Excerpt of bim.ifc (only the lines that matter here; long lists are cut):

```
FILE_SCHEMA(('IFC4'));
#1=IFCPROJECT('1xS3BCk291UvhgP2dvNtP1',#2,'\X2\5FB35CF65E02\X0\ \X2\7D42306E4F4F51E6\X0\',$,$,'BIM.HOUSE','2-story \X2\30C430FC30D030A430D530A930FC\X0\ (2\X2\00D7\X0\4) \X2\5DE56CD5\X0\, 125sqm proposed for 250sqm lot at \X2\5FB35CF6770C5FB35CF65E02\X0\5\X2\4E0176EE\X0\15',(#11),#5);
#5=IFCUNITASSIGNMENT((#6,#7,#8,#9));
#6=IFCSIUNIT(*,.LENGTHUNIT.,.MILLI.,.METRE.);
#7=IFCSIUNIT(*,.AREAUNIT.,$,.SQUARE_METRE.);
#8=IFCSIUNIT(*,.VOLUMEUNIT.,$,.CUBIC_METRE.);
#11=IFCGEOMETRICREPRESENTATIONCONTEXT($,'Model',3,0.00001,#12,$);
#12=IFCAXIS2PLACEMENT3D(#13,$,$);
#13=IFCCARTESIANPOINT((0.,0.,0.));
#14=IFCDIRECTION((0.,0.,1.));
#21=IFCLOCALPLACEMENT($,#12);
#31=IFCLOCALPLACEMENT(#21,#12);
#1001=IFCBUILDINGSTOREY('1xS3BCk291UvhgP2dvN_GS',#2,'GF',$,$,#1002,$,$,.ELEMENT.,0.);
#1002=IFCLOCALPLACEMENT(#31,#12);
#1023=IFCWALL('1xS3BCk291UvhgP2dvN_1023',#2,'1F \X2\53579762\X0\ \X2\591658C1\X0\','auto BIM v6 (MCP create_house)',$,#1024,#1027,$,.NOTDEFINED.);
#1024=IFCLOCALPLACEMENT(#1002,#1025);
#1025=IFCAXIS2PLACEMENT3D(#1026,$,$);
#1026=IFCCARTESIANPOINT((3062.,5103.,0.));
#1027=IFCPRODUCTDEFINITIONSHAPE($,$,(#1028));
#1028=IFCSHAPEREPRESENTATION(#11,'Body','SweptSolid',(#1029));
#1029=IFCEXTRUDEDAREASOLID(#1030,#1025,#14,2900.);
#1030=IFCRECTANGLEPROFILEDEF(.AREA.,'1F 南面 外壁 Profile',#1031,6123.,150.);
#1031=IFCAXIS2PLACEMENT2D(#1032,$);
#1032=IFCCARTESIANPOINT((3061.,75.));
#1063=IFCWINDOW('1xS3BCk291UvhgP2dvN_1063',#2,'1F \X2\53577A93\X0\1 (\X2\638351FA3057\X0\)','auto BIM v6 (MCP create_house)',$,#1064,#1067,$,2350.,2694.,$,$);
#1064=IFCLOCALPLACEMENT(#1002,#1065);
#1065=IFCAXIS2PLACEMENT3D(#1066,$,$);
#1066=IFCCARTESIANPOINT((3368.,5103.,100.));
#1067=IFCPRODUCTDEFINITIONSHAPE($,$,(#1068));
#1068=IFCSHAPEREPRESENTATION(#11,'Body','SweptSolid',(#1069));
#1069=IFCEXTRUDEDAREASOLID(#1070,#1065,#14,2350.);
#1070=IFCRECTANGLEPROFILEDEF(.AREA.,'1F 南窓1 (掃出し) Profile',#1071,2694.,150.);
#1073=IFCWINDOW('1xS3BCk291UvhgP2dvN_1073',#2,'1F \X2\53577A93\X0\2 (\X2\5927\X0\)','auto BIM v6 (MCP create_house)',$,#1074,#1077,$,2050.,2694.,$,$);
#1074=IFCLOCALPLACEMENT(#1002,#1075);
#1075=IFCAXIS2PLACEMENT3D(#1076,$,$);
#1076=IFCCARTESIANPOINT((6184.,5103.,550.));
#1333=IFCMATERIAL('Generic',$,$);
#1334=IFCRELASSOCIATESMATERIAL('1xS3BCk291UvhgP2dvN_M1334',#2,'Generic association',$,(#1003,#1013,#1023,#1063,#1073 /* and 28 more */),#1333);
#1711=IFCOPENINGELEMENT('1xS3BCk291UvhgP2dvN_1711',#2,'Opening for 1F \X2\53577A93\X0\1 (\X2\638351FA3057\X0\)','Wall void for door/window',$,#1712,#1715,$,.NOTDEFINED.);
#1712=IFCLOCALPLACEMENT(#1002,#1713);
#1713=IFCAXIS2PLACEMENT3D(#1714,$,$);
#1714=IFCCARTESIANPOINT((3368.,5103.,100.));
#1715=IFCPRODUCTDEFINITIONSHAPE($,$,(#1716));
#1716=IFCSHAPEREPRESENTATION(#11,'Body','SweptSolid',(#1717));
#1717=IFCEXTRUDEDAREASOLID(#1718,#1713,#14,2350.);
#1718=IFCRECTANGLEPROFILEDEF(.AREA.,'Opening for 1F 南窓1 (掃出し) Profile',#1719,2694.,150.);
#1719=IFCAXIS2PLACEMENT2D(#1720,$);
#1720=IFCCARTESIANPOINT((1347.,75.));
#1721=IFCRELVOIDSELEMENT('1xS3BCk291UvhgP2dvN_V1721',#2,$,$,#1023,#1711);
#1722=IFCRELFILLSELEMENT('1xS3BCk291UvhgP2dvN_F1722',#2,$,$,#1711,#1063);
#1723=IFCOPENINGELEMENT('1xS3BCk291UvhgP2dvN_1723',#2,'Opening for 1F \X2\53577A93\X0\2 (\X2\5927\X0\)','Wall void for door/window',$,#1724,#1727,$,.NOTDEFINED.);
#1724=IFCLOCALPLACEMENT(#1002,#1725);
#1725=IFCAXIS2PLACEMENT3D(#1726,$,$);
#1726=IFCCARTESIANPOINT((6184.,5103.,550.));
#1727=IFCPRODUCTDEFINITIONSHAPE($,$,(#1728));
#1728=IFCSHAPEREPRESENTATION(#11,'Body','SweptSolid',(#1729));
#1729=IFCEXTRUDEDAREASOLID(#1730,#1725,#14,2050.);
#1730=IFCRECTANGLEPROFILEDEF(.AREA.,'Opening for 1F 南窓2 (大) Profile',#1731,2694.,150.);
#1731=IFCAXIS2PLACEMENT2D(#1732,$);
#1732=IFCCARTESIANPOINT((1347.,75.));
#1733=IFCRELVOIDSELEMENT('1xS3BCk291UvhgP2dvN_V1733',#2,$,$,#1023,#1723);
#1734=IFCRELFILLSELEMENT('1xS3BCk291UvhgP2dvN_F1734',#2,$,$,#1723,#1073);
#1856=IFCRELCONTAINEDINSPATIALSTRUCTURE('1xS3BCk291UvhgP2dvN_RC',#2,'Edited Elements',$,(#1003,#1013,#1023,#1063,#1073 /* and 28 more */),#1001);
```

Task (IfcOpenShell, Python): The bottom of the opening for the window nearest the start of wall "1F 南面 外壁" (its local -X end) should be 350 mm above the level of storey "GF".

```python
import numpy as np
import ifcopenshell
import ifcopenshell.api.geometry
import ifcopenshell.geom
import ifcopenshell.util.element
import ifcopenshell.util.placement
import ifcopenshell.util.shape
import ifcopenshell.util.unit

model = ifcopenshell.open("bim.ifc")
unit_scale = ifcopenshell.util.unit.calculate_unit_scale(model)

window = model.by_guid("1xS3BCk291UvhgP2dvN_1063")
opening = window.FillsVoids[0].RelatingOpeningElement
storey = ifcopenshell.util.element.get_container(window, ifc_class="IfcBuildingStorey")
level = ifcopenshell.util.placement.get_local_placement(storey.ObjectPlacement)[2, 3]

# The opening's origin need not be at the sill, so measure its lowest point.
shape = ifcopenshell.geom.create_shape(ifcopenshell.geom.settings(), opening)
bottom = ifcopenshell.util.shape.get_shape_bottom_elevation(shape, shape.geometry) / unit_scale
dz = level + 0.35 / unit_scale - bottom

shift = np.array([0.0, 0.0, dz])
# The window is not placed relative to its opening, so move both.
for product in (opening, window):
    matrix = ifcopenshell.util.placement.get_local_placement(product.ObjectPlacement)
    matrix[:3, 3] += shift
    ifcopenshell.api.geometry.edit_object_placement(model, product=product, matrix=matrix, is_si=False)

print(f"moved by {dz * unit_scale:+.3f} m")

model.write("bim-out.ifc")
```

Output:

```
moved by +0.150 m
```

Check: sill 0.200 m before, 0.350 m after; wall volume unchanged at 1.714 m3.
